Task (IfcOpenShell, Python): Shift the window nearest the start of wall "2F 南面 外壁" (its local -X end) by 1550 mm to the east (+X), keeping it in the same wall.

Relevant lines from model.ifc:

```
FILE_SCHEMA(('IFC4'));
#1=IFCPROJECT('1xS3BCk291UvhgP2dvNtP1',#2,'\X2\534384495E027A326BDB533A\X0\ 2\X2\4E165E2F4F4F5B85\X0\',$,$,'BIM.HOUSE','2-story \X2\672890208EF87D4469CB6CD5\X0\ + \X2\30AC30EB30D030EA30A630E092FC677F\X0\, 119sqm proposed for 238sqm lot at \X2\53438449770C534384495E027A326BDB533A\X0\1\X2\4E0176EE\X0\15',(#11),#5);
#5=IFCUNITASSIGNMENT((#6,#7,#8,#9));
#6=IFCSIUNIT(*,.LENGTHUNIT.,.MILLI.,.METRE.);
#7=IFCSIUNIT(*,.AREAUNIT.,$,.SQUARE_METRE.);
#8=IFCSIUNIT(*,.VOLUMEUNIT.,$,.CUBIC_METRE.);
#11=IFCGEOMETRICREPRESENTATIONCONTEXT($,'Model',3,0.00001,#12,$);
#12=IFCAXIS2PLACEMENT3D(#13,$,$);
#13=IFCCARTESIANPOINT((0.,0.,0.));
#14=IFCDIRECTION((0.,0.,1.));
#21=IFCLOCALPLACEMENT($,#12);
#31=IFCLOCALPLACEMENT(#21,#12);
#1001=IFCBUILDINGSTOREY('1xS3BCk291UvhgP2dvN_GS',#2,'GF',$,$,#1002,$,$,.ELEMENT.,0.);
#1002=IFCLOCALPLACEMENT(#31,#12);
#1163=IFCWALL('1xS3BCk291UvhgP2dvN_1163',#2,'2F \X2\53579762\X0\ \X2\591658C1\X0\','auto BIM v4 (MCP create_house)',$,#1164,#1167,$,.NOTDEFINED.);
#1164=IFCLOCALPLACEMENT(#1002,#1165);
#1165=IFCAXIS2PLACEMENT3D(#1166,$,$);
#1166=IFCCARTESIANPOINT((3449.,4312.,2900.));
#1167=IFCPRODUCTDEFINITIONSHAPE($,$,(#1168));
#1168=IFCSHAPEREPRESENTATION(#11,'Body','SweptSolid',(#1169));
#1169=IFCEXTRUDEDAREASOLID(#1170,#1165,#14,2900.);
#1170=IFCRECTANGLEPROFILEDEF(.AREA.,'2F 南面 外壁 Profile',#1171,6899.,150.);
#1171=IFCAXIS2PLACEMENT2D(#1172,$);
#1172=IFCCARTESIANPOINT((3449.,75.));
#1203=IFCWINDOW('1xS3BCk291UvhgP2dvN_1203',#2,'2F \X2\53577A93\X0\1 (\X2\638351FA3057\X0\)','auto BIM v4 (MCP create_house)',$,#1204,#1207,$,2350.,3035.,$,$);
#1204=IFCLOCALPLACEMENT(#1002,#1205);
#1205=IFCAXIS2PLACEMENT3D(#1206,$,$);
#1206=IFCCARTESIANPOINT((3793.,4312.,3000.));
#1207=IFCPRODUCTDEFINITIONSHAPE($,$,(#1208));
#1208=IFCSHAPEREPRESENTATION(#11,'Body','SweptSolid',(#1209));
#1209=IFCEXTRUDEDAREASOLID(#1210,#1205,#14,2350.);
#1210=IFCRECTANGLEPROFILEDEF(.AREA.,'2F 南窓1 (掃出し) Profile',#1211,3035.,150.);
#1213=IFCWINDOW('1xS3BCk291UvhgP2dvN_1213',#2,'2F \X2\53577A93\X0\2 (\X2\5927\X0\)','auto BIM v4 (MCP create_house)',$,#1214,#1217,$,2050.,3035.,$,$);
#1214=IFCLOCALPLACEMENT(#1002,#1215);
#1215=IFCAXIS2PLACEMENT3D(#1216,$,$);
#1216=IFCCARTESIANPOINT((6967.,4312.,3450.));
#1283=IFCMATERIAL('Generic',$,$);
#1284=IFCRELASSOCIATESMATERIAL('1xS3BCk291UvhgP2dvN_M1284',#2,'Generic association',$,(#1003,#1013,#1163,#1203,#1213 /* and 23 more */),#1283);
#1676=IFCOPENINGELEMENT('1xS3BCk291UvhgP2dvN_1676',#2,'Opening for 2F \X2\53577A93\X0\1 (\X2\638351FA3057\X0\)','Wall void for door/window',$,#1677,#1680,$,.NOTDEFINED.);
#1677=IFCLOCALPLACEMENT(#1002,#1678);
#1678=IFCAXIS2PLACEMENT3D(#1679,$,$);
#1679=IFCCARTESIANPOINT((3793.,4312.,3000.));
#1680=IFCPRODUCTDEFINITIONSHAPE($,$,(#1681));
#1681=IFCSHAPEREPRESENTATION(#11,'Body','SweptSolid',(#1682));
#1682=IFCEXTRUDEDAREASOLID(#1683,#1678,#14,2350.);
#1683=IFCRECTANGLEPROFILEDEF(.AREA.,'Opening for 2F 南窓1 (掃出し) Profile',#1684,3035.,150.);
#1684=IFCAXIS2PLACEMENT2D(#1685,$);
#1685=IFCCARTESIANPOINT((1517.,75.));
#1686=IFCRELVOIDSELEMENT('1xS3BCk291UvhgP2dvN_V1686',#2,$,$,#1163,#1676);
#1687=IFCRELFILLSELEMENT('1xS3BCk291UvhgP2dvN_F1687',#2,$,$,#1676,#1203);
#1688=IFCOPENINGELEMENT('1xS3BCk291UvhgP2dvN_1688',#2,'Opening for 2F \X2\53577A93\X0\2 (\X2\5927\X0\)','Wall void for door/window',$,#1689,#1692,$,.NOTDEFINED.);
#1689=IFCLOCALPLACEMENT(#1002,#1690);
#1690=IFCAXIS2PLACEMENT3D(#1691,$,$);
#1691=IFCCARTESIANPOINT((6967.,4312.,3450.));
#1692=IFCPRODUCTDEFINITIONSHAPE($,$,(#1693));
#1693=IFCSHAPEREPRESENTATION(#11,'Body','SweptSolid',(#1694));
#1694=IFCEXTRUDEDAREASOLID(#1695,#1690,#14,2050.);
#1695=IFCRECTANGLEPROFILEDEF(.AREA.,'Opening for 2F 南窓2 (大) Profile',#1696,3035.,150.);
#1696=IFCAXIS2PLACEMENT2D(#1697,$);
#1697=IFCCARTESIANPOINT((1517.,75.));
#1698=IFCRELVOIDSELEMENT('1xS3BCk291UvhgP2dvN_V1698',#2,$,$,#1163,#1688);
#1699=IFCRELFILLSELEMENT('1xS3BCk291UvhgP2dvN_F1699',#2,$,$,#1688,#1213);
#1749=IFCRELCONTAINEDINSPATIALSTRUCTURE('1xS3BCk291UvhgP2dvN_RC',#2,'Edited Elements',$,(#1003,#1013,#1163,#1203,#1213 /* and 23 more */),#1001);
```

```python
import ifcopenshell
import ifcopenshell.api.geometry
import ifcopenshell.util.placement
import ifcopenshell.util.unit

model = ifcopenshell.open("model.ifc")
unit_scale = ifcopenshell.util.unit.calculate_unit_scale(model)

window = model.by_guid("1xS3BCk291UvhgP2dvN_1203")
opening = window.FillsVoids[0].RelatingOpeningElement
wall = opening.VoidsElements[0].RelatingBuildingElement

wall_matrix = ifcopenshell.util.placement.get_local_placement(wall.ObjectPlacement)
shift = wall_matrix[:3, 0] * 1.55 / unit_scale
before = ifcopenshell.util.placement.get_local_placement(window.ObjectPlacement)[:3, 3].copy()

# The window is not placed relative to its opening, so move both.
for product in (opening, window):
    matrix = ifcopenshell.util.placement.get_local_placement(product.ObjectPlacement)
    matrix[:3, 3] += shift
    ifcopenshell.api.geometry.edit_object_placement(model, product=product, matrix=matrix, is_si=False)

after = ifcopenshell.util.placement.get_local_placement(window.ObjectPlacement)[:3, 3]
print("window moved by", (after - before).round(3) + 0.0)

model.write("model_edited.ifc")
```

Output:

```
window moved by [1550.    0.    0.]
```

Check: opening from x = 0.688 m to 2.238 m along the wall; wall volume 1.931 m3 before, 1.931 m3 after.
